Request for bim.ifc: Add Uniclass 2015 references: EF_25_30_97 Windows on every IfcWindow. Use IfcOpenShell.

First a look at what the model holds.

```python
import ifcopenshell

model = ifcopenshell.open("bim.ifc")
print(model.schema)
print("classifications:", [c.Name for c in model.by_type("IfcClassification")])
for ifc_class in ("IfcDoor", "IfcRoof", "IfcStair", "IfcWall", "IfcWindow"):
    print(ifc_class, len(model.by_type(ifc_class)))
```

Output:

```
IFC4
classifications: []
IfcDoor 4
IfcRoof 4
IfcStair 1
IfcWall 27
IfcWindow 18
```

```python
import ifcopenshell
import ifcopenshell.api.classification

model = ifcopenshell.open("bim.ifc")

system = ifcopenshell.api.classification.add_classification(model, classification="Uniclass 2015")

codes = {
    "IfcWindow": ("EF_25_30_97", "Windows"),
}
for ifc_class, (code, name) in codes.items():
    products = model.by_type(ifc_class)
    ifcopenshell.api.classification.add_reference(
        model, products=products, classification=system, identification=code, name=name
    )
    print(code, len(products))

model.write("bim_rev.ifc")
```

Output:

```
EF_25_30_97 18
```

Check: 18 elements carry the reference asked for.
